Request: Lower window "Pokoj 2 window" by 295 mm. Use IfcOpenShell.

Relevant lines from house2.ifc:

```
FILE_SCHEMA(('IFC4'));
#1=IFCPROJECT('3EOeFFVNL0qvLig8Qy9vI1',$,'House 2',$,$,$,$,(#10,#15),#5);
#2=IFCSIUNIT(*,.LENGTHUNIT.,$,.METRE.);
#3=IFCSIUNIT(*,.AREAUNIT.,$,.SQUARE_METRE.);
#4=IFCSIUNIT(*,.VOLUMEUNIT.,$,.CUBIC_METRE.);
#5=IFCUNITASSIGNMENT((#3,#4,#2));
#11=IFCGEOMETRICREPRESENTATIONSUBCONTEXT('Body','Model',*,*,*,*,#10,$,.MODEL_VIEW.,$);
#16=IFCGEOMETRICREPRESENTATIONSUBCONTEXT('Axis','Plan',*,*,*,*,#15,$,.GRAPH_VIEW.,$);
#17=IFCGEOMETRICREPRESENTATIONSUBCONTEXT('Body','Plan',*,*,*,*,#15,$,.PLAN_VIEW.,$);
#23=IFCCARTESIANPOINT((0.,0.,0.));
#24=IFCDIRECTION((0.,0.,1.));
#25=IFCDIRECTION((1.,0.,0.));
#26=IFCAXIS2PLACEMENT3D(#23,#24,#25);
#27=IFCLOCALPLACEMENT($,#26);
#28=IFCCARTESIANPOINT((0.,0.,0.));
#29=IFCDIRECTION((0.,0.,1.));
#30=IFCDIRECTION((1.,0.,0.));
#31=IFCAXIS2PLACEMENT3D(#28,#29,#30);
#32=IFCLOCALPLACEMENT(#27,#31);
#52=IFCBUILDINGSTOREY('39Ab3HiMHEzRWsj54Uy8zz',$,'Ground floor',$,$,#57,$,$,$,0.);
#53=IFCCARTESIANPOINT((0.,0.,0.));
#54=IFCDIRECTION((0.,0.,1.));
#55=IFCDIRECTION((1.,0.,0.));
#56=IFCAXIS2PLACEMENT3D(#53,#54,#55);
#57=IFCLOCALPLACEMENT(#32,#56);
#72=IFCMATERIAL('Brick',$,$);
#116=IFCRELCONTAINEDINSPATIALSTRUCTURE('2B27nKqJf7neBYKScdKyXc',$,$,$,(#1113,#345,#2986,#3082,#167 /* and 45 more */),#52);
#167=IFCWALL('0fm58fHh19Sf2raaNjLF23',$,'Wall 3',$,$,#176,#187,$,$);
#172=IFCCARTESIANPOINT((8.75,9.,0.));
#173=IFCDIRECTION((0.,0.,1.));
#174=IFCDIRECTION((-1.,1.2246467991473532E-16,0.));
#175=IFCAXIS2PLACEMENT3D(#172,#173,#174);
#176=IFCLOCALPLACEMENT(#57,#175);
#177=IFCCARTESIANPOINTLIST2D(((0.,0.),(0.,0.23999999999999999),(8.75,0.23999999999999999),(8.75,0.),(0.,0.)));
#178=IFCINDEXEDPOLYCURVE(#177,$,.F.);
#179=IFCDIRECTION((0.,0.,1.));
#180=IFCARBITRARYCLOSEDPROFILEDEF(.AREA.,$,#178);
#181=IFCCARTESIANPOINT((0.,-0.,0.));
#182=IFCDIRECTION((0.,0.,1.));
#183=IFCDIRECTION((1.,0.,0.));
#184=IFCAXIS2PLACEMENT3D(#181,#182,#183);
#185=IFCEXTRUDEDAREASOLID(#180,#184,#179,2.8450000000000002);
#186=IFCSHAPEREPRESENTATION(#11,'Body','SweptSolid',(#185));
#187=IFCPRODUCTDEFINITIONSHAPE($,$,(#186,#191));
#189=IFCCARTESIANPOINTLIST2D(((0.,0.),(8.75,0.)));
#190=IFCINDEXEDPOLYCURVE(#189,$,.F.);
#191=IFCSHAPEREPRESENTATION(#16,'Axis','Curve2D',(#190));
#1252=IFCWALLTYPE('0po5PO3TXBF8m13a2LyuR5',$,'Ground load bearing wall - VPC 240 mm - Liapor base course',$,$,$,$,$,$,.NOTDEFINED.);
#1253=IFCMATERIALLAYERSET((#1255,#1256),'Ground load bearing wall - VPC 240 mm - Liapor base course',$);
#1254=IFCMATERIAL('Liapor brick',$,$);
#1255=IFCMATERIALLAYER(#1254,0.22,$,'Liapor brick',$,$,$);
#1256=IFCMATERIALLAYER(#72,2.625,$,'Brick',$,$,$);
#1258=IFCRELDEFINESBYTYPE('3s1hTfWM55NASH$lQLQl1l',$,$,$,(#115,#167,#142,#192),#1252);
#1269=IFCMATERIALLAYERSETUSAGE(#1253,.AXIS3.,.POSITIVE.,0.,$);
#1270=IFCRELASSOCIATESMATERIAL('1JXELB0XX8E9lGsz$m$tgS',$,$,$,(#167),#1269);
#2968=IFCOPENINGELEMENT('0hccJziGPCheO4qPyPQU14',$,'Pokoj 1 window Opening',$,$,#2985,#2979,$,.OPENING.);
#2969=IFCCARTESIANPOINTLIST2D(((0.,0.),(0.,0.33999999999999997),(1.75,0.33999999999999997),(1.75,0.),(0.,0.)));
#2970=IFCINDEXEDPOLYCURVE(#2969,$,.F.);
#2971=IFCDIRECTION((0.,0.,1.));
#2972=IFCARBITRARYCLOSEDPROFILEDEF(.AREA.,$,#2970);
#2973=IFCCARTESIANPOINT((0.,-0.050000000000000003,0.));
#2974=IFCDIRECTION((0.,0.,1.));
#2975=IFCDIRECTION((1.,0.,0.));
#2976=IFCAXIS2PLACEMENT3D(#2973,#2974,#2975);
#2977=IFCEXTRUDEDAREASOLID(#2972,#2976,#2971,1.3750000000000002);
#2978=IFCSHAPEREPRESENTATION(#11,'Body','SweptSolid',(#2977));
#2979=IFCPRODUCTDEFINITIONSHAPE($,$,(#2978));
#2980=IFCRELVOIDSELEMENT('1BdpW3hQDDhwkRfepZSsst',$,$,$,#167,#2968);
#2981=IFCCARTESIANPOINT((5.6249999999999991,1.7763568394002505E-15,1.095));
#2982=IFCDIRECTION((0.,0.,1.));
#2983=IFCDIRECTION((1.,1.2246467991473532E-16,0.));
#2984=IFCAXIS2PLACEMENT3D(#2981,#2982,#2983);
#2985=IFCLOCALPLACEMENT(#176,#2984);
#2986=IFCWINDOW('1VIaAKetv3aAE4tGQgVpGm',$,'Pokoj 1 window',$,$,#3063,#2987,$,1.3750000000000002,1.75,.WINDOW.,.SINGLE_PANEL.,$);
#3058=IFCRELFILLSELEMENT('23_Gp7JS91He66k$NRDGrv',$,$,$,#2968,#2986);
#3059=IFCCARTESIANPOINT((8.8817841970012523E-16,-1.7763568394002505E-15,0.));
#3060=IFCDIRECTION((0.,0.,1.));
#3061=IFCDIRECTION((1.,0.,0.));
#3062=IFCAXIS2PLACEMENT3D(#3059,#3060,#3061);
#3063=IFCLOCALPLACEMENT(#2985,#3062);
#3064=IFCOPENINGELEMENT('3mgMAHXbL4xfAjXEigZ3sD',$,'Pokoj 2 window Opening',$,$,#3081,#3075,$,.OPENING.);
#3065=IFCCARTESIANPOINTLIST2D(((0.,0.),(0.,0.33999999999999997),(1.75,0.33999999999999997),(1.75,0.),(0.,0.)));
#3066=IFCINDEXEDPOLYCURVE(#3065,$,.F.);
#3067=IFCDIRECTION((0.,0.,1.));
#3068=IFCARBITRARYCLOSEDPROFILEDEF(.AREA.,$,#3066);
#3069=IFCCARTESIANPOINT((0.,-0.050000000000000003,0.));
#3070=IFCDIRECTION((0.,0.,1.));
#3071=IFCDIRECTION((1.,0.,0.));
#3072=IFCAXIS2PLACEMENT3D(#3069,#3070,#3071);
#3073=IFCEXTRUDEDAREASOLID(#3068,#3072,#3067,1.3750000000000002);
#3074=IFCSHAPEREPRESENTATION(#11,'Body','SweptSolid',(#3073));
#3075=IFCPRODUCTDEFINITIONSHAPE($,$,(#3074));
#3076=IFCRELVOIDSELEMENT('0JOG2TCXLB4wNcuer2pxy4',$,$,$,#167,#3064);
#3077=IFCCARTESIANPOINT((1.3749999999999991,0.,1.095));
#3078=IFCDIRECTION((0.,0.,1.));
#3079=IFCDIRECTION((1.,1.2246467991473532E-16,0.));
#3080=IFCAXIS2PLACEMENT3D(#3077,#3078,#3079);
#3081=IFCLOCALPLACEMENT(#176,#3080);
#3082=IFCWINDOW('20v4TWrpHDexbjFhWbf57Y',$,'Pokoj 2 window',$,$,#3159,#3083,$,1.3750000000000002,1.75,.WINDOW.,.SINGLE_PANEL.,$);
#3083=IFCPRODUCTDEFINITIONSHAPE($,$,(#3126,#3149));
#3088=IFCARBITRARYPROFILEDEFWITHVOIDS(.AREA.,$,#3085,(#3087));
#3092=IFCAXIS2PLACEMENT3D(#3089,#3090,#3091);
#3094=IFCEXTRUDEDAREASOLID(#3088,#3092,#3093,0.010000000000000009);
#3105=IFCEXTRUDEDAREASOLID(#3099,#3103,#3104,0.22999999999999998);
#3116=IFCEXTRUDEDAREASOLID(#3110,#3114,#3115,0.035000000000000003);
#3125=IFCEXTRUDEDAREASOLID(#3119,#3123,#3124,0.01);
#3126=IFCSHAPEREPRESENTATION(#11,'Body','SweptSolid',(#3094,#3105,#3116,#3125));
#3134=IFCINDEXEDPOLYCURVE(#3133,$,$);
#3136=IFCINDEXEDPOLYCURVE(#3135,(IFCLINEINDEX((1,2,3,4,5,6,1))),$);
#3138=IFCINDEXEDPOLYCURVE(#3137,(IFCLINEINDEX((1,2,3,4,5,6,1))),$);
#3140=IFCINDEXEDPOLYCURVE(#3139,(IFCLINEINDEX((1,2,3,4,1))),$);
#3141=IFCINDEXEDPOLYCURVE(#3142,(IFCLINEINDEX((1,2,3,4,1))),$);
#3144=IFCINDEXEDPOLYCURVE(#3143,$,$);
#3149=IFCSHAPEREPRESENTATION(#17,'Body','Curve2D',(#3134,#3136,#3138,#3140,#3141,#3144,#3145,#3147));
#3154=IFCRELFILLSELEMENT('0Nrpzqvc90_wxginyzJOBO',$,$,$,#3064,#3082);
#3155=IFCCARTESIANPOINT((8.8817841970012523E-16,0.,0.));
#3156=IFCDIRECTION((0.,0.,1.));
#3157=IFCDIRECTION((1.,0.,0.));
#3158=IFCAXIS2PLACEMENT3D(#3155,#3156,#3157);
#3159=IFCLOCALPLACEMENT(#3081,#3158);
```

```python
import numpy as np
import ifcopenshell
import ifcopenshell.api.geometry
import ifcopenshell.util.placement
import ifcopenshell.util.unit

model = ifcopenshell.open("house2.ifc")
unit_scale = ifcopenshell.util.unit.calculate_unit_scale(model)

window = model.by_id(3082)
opening = window.FillsVoids[0].RelatingOpeningElement
dz = -0.295 / unit_scale

shift = np.array([0.0, 0.0, dz])
# The window is placed relative to its opening, so it follows when the opening moves.
matrix = ifcopenshell.util.placement.get_local_placement(opening.ObjectPlacement)
matrix[:3, 3] += shift
ifcopenshell.api.geometry.edit_object_placement(
    model, product=opening, matrix=matrix, is_si=False, should_transform_children=True
)

print(f"moved by {dz * unit_scale:+.3f} m")

model.write("house2-out.ifc")
```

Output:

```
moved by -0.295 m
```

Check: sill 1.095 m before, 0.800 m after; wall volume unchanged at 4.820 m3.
